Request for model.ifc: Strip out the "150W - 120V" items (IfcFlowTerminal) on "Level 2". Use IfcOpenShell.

First a look at what the model holds.

```python
import ifcopenshell
import ifcopenshell.util.element

model = ifcopenshell.open("model.ifc")
print(model.schema)
storey = next(s for s in model.by_type("IfcBuildingStorey") if s.Name == "Level 2")
terminals = [e for e in ifcopenshell.util.element.get_decomposition(storey) if e.is_a("IfcFlowTerminal")]
seen = {}
for e in terminals:
    element_type = ifcopenshell.util.element.get_type(e)
    name = element_type.Name if element_type not in (None, e) else None
    seen[name] = seen.get(name, 0) + 1
for name, count in sorted(seen.items(), key=str):
    print(count, "x", name)
```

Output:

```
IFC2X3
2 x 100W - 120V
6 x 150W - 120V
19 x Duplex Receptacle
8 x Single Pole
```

```python
import ifcopenshell
import ifcopenshell.api.root
import ifcopenshell.util.element

model = ifcopenshell.open("model.ifc")

storey = next(s for s in model.by_type("IfcBuildingStorey") if s.Name == "Level 2")
terminals = [e for e in ifcopenshell.util.element.get_decomposition(storey) if e.is_a("IfcFlowTerminal")]
targets = [e for e in terminals if (t := ifcopenshell.util.element.get_type(e)) not in (None, e) and t.Name == "150W - 120V"]

for e in targets:
    ifcopenshell.api.root.remove_product(model, product=e)
print(len(targets), "removed")

model.write("model_updated.ifc")
```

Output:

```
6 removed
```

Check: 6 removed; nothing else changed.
